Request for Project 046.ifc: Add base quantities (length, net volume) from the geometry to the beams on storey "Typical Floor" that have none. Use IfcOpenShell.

First a look at what the model holds.

```python
import ifcopenshell
import ifcopenshell.util.element
import ifcopenshell.util.unit

model = ifcopenshell.open("Project 046.ifc")
print(model.schema)
for unit_type in ("LENGTHUNIT", "AREAUNIT", "VOLUMEUNIT"):
    print(unit_type, ifcopenshell.util.unit.calculate_unit_scale(model, unit_type))
storey = next(s for s in model.by_type("IfcBuildingStorey") if s.Name == "Typical Floor")
beams = [e for e in ifcopenshell.util.element.get_decomposition(storey) if e.is_a("IfcBeam")]
for e in sorted(beams, key=lambda e: e.id()):
    print(e.id(), e.is_a(), e.Name, list(ifcopenshell.util.element.get_psets(e, qtos_only=True)), sep=" | ")
```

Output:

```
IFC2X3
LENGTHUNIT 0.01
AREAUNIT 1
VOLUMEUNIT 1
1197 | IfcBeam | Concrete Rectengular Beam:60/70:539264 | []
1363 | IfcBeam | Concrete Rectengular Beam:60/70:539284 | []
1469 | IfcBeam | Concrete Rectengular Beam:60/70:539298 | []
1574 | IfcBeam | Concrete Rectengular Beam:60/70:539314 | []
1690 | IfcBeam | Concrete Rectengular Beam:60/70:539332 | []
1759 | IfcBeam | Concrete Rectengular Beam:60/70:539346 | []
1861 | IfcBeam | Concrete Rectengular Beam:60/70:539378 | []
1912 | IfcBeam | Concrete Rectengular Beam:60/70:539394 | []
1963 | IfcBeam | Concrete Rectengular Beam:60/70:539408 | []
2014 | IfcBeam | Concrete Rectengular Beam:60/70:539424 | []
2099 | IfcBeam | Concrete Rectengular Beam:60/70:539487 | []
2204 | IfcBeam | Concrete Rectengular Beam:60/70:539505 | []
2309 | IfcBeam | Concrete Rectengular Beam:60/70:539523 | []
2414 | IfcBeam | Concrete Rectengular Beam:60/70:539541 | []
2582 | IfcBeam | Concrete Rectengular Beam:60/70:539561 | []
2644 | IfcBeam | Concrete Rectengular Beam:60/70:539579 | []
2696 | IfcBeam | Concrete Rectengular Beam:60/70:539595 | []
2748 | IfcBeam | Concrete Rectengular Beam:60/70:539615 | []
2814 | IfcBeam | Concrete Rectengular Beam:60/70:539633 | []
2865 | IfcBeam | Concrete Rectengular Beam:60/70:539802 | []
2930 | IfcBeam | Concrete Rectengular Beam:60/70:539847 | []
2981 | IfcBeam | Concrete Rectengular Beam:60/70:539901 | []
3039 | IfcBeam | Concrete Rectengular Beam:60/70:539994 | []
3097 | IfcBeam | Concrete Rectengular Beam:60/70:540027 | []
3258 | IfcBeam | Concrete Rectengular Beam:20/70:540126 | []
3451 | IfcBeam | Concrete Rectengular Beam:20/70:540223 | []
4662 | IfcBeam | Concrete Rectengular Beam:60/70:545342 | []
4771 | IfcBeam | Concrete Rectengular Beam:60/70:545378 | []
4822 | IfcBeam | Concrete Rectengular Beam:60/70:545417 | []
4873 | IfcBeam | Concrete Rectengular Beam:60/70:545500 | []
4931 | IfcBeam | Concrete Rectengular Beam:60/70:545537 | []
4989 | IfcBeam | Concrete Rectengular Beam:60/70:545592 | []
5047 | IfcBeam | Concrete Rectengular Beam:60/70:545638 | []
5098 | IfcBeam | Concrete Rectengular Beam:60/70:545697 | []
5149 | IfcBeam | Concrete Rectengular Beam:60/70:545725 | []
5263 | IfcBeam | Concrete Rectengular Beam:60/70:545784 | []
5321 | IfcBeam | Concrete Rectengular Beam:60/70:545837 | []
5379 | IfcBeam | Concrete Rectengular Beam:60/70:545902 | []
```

```python
import ifcopenshell
import ifcopenshell.api.pset
import ifcopenshell.geom
import ifcopenshell.util.element
import ifcopenshell.util.shape
import ifcopenshell.util.unit

model = ifcopenshell.open("Project 046.ifc")
unit_scale = ifcopenshell.util.unit.calculate_unit_scale(model)
volume_scale = ifcopenshell.util.unit.calculate_unit_scale(model, "VOLUMEUNIT")
settings = ifcopenshell.geom.settings()

storey = next(s for s in model.by_type("IfcBuildingStorey") if s.Name == "Typical Floor")
beams = [e for e in ifcopenshell.util.element.get_decomposition(storey) if e.is_a("IfcBeam")]

for e in sorted(beams, key=lambda e: e.id()):
    if ifcopenshell.util.element.get_psets(e, qtos_only=True, should_inherit=False):
        continue
    # Geometry comes back in metres, in the element's own axes.
    shape = ifcopenshell.geom.create_shape(settings, e)
    values = {
        "Length": ifcopenshell.util.shape.get_max_xyz(shape.geometry) / unit_scale,
        "NetVolume": ifcopenshell.util.shape.get_volume(shape.geometry) / volume_scale,
    }
    qto = ifcopenshell.api.pset.add_qto(model, product=e, name="BaseQuantities")
    ifcopenshell.api.pset.edit_qto(model, qto=qto, properties=values)
    print(e.id(), {k: round(v, 3) for k, v in values.items()})

model.write("Project 046_rev.ifc")
```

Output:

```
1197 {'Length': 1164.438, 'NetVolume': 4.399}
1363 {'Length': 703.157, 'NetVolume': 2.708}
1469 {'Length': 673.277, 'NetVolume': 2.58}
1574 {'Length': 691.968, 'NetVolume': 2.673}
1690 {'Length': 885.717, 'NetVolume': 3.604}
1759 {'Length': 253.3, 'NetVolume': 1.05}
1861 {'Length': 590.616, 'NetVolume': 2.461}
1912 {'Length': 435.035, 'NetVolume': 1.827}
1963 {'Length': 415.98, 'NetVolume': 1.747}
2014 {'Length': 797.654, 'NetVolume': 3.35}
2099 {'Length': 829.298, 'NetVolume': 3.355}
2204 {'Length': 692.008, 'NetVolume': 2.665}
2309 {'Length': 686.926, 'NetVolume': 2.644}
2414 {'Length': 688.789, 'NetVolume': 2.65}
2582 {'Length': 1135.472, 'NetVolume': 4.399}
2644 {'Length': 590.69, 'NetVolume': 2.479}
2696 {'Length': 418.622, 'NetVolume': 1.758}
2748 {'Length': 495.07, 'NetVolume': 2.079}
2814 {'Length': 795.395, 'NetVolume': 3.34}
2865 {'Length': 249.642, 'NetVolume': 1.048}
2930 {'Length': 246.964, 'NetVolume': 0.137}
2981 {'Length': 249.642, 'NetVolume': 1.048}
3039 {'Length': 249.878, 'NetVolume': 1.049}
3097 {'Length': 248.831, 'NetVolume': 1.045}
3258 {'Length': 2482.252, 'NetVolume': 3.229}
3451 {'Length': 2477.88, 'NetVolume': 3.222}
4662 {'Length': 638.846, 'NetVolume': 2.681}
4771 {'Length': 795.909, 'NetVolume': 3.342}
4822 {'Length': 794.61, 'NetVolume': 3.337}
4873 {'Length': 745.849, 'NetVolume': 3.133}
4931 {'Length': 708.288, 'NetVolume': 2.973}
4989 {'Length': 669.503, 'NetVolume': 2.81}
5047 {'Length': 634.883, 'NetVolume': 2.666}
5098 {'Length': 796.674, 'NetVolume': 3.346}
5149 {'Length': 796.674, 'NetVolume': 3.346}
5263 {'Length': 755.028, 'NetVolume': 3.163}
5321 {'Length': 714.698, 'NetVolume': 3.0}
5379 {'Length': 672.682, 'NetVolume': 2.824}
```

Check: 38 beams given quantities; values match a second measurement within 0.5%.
